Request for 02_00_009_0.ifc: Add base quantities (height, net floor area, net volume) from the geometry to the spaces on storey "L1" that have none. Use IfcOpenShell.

First a look at what the model holds.

```python
import ifcopenshell
import ifcopenshell.util.element
import ifcopenshell.util.unit

model = ifcopenshell.open("02_00_009_0.ifc")
print(model.schema)
for unit_type in ("LENGTHUNIT", "AREAUNIT", "VOLUMEUNIT"):
    print(unit_type, ifcopenshell.util.unit.calculate_unit_scale(model, unit_type))
storey = next(s for s in model.by_type("IfcBuildingStorey") if s.Name == "L1")
spaces = [e for e in ifcopenshell.util.element.get_decomposition(storey) if e.is_a("IfcSpace")]
for e in sorted(spaces, key=lambda e: e.id()):
    print(e.id(), e.is_a(), e.Name, list(ifcopenshell.util.element.get_psets(e, qtos_only=True)), sep=" | ")
```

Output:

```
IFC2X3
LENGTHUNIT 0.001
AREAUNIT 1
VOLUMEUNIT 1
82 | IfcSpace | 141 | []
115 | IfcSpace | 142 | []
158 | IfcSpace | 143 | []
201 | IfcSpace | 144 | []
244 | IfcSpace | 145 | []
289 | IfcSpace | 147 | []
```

```python
import ifcopenshell
import ifcopenshell.api.pset
import ifcopenshell.geom
import ifcopenshell.util.element
import ifcopenshell.util.shape
import ifcopenshell.util.unit

model = ifcopenshell.open("02_00_009_0.ifc")
unit_scale = ifcopenshell.util.unit.calculate_unit_scale(model)
area_scale = ifcopenshell.util.unit.calculate_unit_scale(model, "AREAUNIT")
volume_scale = ifcopenshell.util.unit.calculate_unit_scale(model, "VOLUMEUNIT")
settings = ifcopenshell.geom.settings()

storey = next(s for s in model.by_type("IfcBuildingStorey") if s.Name == "L1")
spaces = [e for e in ifcopenshell.util.element.get_decomposition(storey) if e.is_a("IfcSpace")]

for e in sorted(spaces, key=lambda e: e.id()):
    if ifcopenshell.util.element.get_psets(e, qtos_only=True, should_inherit=False):
        continue
    # Geometry comes back in metres, in the element's own axes.
    shape = ifcopenshell.geom.create_shape(settings, e)
    values = {
        "Height": ifcopenshell.util.shape.get_z(shape.geometry) / unit_scale,
        "NetFloorArea": ifcopenshell.util.shape.get_footprint_area(shape.geometry) / area_scale,
        "NetVolume": ifcopenshell.util.shape.get_volume(shape.geometry) / volume_scale,
    }
    qto = ifcopenshell.api.pset.add_qto(model, product=e, name="BaseQuantities")
    ifcopenshell.api.pset.edit_qto(model, qto=qto, properties=values)
    print(e.id(), {k: round(v, 3) for k, v in values.items()})

model.write("02_00_009_0-out.ifc")
```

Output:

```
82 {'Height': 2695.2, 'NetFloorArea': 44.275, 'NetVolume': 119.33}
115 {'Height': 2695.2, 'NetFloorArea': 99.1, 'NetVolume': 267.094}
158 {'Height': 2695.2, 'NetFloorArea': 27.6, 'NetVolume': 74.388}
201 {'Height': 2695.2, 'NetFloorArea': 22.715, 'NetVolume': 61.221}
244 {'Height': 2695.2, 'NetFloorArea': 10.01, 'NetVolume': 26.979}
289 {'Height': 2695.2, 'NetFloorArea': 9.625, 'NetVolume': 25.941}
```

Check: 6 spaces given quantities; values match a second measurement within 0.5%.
